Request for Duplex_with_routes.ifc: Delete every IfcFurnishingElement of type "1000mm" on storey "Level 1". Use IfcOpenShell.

First a look at what the model holds.

```python
import ifcopenshell
import ifcopenshell.util.element

model = ifcopenshell.open("Duplex_with_routes.ifc")
print(model.schema)
storey = next(s for s in model.by_type("IfcBuildingStorey") if s.Name == "Level 1")
furniture = [e for e in ifcopenshell.util.element.get_decomposition(storey) if e.is_a("IfcFurnishingElement")]
seen = {}
for e in furniture:
    element_type = ifcopenshell.util.element.get_type(e)
    name = element_type.Name if element_type not in (None, e) else None
    seen[name] = seen.get(name, 0) + 1
for name, count in sorted(seen.items(), key=str):
    print(count, "x", name)
```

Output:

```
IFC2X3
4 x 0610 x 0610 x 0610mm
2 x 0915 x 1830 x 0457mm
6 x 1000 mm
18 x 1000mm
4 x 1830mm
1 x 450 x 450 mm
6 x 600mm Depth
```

```python
import ifcopenshell
import ifcopenshell.api.root
import ifcopenshell.util.element

model = ifcopenshell.open("Duplex_with_routes.ifc")

storey = next(s for s in model.by_type("IfcBuildingStorey") if s.Name == "Level 1")
furniture = [e for e in ifcopenshell.util.element.get_decomposition(storey) if e.is_a("IfcFurnishingElement")]
targets = [e for e in furniture if (t := ifcopenshell.util.element.get_type(e)) not in (None, e) and t.Name == "1000mm"]

for e in targets:
    ifcopenshell.api.root.remove_product(model, product=e)
print(len(targets), "removed")

model.write("Duplex_with_routes_rev.ifc")
```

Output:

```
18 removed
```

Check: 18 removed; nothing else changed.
